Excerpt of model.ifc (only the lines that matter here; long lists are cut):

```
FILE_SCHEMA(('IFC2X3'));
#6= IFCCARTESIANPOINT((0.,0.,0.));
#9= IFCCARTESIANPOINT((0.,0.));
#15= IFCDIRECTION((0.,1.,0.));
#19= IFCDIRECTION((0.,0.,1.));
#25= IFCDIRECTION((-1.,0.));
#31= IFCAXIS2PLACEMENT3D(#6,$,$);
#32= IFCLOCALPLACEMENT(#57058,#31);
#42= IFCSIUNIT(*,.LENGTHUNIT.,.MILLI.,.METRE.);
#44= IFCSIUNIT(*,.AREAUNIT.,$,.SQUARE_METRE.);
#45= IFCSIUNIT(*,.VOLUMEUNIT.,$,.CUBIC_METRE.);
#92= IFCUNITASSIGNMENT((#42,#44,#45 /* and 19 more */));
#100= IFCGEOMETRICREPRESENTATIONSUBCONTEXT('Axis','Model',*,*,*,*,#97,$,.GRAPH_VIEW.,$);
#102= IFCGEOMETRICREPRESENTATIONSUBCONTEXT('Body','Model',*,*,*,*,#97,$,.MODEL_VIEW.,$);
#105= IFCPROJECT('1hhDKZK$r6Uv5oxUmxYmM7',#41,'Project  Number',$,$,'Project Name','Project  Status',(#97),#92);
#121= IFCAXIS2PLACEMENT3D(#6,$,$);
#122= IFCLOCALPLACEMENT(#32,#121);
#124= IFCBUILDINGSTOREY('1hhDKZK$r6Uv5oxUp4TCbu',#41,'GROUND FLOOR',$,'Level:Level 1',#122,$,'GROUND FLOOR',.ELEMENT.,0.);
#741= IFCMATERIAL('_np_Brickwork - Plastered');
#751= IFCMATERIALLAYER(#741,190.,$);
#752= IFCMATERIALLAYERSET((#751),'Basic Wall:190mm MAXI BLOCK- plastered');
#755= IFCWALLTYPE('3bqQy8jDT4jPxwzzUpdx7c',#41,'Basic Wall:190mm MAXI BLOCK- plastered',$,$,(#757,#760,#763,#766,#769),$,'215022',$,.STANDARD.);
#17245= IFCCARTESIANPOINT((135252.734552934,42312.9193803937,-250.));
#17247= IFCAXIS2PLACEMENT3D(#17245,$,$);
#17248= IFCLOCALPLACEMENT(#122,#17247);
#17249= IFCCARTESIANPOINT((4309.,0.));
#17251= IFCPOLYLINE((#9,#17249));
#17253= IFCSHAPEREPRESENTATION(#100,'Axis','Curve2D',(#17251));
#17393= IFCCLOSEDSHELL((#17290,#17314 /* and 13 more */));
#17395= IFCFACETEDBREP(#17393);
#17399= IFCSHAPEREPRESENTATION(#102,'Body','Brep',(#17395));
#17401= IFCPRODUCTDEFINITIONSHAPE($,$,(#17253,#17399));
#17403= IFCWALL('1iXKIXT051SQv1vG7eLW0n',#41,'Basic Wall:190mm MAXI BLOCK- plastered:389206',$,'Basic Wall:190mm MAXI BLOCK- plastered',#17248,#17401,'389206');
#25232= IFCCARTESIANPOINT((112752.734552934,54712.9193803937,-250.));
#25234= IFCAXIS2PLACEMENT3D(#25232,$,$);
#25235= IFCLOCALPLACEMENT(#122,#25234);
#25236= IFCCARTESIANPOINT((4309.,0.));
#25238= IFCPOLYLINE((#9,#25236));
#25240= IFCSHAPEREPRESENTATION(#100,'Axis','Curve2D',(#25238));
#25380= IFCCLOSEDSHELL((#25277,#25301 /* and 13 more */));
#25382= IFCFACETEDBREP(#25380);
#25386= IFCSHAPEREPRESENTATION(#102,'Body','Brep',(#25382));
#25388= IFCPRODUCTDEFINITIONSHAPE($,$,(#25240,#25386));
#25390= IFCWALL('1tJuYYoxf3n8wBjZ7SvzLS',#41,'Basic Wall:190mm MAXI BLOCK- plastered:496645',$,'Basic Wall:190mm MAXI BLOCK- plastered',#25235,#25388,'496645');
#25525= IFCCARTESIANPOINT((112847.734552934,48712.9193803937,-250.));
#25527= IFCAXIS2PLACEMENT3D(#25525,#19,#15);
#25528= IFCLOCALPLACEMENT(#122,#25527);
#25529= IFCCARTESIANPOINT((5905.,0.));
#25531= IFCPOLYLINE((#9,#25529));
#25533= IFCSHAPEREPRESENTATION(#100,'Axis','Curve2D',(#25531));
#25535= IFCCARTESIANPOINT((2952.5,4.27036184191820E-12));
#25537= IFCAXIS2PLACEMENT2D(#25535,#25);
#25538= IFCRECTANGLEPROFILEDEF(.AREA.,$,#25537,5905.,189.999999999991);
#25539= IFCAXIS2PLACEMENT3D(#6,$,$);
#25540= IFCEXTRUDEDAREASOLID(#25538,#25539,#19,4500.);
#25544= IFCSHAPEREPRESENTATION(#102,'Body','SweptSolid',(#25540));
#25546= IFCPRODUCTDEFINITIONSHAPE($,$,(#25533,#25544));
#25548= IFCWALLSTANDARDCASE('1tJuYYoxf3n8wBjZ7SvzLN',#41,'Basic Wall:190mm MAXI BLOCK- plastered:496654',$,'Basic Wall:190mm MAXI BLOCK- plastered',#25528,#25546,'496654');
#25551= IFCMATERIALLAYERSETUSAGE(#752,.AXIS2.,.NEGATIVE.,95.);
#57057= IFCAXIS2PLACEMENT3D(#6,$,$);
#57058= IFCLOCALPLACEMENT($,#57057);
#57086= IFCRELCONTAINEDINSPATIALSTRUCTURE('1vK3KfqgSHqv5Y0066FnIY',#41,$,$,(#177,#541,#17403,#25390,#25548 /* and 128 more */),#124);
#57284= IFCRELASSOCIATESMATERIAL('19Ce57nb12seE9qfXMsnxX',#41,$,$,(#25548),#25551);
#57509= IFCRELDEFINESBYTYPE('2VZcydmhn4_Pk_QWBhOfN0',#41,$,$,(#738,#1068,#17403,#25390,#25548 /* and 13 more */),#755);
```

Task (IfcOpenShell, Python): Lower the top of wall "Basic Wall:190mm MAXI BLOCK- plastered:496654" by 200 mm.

```python
import ifcopenshell
import ifcopenshell.geom
import ifcopenshell.util.representation
import ifcopenshell.util.shape

model = ifcopenshell.open("model.ifc")
settings = ifcopenshell.geom.settings()


def volume(element):
    """Net volume in cubic metres, openings subtracted."""
    shape = ifcopenshell.geom.create_shape(settings, element)
    return ifcopenshell.util.shape.get_volume(shape.geometry)


wall = model.by_guid("1tJuYYoxf3n8wBjZ7SvzLN")
before = volume(wall)

body = ifcopenshell.util.representation.get_representation(wall, "Model", "Body")
solid = body.Items[0]
old_height = solid.Depth
solid.Depth -= 200.0
after = volume(wall)

print(f"height {old_height:g} -> {solid.Depth:g}, volume {before:.3f} -> {after:.3f} m3")

model.write("model_v2.ifc")
```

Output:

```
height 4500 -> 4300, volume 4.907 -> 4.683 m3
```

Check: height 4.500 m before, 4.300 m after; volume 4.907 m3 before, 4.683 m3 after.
